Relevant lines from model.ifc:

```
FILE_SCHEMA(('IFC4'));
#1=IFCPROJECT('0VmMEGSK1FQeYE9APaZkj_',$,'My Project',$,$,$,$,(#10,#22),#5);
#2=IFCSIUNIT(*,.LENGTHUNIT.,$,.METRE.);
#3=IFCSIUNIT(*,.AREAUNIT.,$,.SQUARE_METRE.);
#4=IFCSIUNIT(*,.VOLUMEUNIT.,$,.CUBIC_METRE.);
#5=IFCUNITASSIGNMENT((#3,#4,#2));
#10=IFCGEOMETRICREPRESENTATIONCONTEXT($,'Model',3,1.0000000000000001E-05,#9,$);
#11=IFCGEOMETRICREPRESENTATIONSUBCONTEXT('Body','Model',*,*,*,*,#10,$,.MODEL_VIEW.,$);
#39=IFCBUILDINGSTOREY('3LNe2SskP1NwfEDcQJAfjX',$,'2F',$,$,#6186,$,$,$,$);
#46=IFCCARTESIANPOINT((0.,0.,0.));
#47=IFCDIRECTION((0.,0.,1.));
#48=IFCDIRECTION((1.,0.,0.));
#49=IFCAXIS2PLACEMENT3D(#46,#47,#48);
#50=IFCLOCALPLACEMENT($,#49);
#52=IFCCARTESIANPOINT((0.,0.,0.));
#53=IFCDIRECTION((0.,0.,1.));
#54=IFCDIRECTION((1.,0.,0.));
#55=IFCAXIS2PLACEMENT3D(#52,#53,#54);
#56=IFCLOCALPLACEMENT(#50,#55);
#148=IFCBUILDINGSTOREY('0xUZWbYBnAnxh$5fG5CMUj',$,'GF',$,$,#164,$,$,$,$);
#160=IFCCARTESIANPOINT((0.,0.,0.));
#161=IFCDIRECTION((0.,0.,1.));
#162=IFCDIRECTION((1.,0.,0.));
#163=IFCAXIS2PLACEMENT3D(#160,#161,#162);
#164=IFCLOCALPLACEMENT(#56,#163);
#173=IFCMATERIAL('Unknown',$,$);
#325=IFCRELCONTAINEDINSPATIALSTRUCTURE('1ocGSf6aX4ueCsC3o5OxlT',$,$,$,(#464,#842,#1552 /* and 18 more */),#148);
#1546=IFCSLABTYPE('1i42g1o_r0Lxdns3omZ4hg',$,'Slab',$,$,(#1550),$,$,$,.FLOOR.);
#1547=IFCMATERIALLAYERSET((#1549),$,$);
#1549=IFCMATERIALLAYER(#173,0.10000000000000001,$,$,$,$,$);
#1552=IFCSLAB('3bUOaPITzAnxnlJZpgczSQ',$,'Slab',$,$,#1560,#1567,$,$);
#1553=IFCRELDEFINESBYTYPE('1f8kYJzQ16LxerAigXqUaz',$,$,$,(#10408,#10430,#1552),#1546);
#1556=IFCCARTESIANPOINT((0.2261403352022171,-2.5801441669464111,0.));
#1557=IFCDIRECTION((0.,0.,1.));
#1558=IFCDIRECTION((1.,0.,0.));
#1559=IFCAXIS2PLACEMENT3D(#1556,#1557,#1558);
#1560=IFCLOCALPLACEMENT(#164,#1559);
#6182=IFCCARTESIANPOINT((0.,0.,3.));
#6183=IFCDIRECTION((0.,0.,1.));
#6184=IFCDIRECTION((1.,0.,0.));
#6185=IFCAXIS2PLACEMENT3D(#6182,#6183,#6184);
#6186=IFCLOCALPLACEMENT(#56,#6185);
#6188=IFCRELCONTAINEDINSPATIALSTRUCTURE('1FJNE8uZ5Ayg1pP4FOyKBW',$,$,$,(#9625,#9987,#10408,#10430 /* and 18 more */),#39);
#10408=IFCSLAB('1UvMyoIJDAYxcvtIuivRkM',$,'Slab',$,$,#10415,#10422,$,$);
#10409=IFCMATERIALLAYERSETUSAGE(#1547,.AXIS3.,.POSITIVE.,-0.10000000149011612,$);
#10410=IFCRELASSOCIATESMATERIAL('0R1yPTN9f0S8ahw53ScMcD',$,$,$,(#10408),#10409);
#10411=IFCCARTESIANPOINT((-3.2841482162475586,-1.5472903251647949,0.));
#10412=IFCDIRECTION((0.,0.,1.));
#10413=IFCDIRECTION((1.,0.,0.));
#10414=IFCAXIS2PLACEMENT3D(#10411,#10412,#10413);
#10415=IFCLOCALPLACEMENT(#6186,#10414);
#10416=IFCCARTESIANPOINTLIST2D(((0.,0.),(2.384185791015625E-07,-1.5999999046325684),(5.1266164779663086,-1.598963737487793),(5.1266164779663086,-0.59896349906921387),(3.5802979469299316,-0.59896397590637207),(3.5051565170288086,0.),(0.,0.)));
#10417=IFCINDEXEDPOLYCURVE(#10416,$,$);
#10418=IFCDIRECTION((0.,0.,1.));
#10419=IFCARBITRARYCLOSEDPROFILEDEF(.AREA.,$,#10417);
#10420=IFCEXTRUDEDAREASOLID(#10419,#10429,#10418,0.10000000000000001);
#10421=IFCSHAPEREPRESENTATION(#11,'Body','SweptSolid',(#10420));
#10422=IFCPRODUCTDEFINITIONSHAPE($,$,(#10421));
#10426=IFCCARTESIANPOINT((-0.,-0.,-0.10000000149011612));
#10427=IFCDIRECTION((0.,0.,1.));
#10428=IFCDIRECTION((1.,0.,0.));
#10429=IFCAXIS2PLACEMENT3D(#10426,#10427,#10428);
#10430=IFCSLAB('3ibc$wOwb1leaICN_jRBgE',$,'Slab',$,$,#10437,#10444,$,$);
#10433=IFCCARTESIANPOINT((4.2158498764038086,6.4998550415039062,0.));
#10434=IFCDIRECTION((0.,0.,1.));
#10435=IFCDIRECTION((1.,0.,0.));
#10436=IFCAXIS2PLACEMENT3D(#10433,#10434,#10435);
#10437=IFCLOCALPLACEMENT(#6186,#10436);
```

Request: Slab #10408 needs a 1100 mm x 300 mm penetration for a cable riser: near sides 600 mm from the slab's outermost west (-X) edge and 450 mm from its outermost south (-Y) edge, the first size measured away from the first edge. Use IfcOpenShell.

```python
import numpy as np
import ifcopenshell
import ifcopenshell.api.feature
import ifcopenshell.api.geometry
import ifcopenshell.api.root
import ifcopenshell.geom
import ifcopenshell.util.placement
import ifcopenshell.util.representation
import ifcopenshell.util.shape
import ifcopenshell.util.unit

model = ifcopenshell.open("model.ifc")
unit_scale = ifcopenshell.util.unit.calculate_unit_scale(model)
settings = ifcopenshell.geom.settings()


def volume(element):
    """Net volume in cubic metres, openings subtracted."""
    shape = ifcopenshell.geom.create_shape(settings, element)
    return ifcopenshell.util.shape.get_volume(shape.geometry)


slab = model.by_id(10408)
before = volume(slab)

# Extent in the slab's own axes, in metres. The edges named are its -X and -Y sides.
slab_shape = ifcopenshell.geom.create_shape(settings, slab)
vertices = ifcopenshell.util.shape.get_vertices(slab_shape.geometry)
x_min, y_min, bottom = vertices.min(axis=0)
top = vertices[:, 2].max()

opening = ifcopenshell.api.root.create_entity(model, ifc_class="IfcOpeningElement", name="Cable riser opening", predefined_type="OPENING")
context = ifcopenshell.util.representation.get_context(model, "Model", "Body", "MODEL_VIEW")
width, depth = 1.1, 0.3
outline = [(0.0, 0.0), (width, 0.0), (width, depth), (0.0, depth), (0.0, 0.0)]
# Overshoot both faces by 50 mm so the cut is clean.
shape = ifcopenshell.api.geometry.add_slab_representation(
    model, context=context, depth=top - bottom + 0.1, polyline=outline
)
ifcopenshell.api.geometry.assign_representation(model, product=opening, representation=shape)

matrix = ifcopenshell.util.placement.get_local_placement(slab.ObjectPlacement)
matrix[:, 3] = matrix @ np.append(np.array([x_min + 0.6, y_min + 0.45, bottom - 0.05]) / unit_scale, 1.0)
ifcopenshell.api.geometry.edit_object_placement(model, product=opening, matrix=matrix, is_si=False)
ifcopenshell.api.feature.add_feature(model, feature=opening, element=slab)

after = volume(slab)

print(f"slab volume {before:.3f} -> {after:.3f} m3")

model.write("model-out.ifc")
```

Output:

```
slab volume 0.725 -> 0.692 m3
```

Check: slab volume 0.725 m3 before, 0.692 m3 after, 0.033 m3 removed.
